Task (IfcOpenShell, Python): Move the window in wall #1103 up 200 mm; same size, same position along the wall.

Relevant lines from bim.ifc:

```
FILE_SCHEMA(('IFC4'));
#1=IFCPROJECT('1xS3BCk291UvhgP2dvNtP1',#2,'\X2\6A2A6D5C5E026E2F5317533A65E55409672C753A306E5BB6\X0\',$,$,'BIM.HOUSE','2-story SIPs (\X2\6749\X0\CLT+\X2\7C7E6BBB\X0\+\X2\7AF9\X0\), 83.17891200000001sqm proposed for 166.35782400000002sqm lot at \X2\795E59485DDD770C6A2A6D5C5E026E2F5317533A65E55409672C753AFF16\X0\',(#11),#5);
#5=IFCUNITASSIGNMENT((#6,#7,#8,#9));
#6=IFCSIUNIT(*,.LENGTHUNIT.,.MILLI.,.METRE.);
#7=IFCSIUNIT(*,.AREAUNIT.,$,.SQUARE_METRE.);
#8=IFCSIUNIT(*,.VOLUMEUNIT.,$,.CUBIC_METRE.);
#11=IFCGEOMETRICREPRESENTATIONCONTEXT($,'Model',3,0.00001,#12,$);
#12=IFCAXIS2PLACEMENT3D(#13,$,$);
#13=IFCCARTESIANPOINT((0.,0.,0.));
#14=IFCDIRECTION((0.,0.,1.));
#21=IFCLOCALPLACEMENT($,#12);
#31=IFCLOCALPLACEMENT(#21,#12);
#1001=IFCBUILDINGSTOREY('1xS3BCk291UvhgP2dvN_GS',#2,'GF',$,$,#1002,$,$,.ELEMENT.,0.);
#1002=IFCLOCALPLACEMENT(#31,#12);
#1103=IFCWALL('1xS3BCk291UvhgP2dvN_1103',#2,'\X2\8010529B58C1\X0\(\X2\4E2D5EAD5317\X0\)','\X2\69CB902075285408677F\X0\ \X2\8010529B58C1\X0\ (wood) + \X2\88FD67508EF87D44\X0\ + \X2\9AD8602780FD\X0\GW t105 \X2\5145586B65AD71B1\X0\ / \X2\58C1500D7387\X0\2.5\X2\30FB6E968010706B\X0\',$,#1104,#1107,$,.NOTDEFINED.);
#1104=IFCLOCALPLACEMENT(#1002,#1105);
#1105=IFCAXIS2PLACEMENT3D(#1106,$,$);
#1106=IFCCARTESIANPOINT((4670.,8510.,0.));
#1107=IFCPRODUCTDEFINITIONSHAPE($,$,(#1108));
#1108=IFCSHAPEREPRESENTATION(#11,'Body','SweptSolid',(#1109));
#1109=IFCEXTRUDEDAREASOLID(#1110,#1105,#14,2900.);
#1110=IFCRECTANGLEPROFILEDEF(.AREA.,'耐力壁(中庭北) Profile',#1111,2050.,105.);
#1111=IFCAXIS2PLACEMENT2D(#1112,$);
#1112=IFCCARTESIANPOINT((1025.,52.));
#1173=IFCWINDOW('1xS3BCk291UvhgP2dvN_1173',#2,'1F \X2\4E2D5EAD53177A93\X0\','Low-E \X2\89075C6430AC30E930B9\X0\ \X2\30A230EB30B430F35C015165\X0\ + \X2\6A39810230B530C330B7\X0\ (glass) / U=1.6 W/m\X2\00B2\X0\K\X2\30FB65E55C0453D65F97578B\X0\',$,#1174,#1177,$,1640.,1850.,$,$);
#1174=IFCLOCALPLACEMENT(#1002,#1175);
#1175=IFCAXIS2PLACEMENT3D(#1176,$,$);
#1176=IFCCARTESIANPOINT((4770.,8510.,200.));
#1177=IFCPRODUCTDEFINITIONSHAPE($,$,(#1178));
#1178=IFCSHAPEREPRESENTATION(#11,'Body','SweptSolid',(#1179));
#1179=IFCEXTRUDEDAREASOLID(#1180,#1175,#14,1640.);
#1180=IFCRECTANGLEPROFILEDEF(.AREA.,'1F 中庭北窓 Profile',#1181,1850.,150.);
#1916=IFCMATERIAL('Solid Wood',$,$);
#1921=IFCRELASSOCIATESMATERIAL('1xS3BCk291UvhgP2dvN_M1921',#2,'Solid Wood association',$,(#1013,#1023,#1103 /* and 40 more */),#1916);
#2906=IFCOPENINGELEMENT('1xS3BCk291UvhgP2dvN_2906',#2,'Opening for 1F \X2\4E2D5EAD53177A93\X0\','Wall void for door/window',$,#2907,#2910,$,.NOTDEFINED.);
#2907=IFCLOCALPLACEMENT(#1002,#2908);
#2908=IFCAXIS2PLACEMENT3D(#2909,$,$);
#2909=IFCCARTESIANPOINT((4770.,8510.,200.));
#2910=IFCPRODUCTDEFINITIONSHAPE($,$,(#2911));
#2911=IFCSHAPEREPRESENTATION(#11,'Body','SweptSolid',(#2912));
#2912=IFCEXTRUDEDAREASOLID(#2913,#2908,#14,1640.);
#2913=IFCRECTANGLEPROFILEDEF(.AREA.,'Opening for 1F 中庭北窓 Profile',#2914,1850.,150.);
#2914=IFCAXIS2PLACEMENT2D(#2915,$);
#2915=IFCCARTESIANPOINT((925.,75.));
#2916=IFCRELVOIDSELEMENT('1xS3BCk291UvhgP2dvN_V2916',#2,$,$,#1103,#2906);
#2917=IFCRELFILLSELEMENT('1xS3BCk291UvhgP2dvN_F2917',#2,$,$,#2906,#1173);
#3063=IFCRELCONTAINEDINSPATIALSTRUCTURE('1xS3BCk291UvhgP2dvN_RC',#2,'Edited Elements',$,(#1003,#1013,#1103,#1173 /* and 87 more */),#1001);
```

```python
import numpy as np
import ifcopenshell
import ifcopenshell.api.geometry
import ifcopenshell.util.placement
import ifcopenshell.util.unit

model = ifcopenshell.open("bim.ifc")
unit_scale = ifcopenshell.util.unit.calculate_unit_scale(model)

window = model.by_guid("1xS3BCk291UvhgP2dvN_1173")
opening = window.FillsVoids[0].RelatingOpeningElement
dz = 0.2 / unit_scale

shift = np.array([0.0, 0.0, dz])
# The window is not placed relative to its opening, so move both.
for product in (opening, window):
    matrix = ifcopenshell.util.placement.get_local_placement(product.ObjectPlacement)
    matrix[:3, 3] += shift
    ifcopenshell.api.geometry.edit_object_placement(model, product=product, matrix=matrix, is_si=False)

print(f"moved by {dz * unit_scale:+.3f} m")

model.write("bim_edited.ifc")
```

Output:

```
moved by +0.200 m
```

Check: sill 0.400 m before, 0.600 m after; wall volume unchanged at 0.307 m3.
